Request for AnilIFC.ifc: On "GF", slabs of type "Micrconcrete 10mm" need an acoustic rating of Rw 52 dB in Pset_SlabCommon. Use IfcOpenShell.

First a look at what the model holds.

```python
import ifcopenshell
import ifcopenshell.util.element

model = ifcopenshell.open("AnilIFC.ifc")
print(model.schema)
storey = next(s for s in model.by_type("IfcBuildingStorey") if s.Name == "GF")
slabs = [e for e in ifcopenshell.util.element.get_decomposition(storey) if e.is_a("IfcSlab")]
seen = {}
for e in slabs:
    element_type = ifcopenshell.util.element.get_type(e)
    key = (element_type.Name if element_type != e and element_type else None, ifcopenshell.util.element.get_pset(e, "Pset_SlabCommon", "AcousticRating"))
    seen[key] = seen.get(key, 0) + 1
for (name, value), count in sorted(seen.items(), key=str):
    print(count, "x", name, "|", value)
```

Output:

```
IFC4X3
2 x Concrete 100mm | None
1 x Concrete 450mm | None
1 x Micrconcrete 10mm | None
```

```python
import ifcopenshell
import ifcopenshell.api.pset
import ifcopenshell.util.element

model = ifcopenshell.open("AnilIFC.ifc")

storey = next(s for s in model.by_type("IfcBuildingStorey") if s.Name == "GF")
slabs = [e for e in ifcopenshell.util.element.get_decomposition(storey) if e.is_a("IfcSlab")]

count = 0
for e in slabs:
    element_type = ifcopenshell.util.element.get_type(e)
    if element_type in (None, e) or element_type.Name != "Micrconcrete 10mm":
        continue
    # add_pset returns the element's existing set when there is one.
    pset = ifcopenshell.api.pset.add_pset(model, product=e, name="Pset_SlabCommon")
    ifcopenshell.api.pset.edit_pset(model, pset=pset, properties={"AcousticRating": "Rw 52 dB"})
    count += 1

print(count, "slabs updated")

model.write("AnilIFC_v2.ifc")
```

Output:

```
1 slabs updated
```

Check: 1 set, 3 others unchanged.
